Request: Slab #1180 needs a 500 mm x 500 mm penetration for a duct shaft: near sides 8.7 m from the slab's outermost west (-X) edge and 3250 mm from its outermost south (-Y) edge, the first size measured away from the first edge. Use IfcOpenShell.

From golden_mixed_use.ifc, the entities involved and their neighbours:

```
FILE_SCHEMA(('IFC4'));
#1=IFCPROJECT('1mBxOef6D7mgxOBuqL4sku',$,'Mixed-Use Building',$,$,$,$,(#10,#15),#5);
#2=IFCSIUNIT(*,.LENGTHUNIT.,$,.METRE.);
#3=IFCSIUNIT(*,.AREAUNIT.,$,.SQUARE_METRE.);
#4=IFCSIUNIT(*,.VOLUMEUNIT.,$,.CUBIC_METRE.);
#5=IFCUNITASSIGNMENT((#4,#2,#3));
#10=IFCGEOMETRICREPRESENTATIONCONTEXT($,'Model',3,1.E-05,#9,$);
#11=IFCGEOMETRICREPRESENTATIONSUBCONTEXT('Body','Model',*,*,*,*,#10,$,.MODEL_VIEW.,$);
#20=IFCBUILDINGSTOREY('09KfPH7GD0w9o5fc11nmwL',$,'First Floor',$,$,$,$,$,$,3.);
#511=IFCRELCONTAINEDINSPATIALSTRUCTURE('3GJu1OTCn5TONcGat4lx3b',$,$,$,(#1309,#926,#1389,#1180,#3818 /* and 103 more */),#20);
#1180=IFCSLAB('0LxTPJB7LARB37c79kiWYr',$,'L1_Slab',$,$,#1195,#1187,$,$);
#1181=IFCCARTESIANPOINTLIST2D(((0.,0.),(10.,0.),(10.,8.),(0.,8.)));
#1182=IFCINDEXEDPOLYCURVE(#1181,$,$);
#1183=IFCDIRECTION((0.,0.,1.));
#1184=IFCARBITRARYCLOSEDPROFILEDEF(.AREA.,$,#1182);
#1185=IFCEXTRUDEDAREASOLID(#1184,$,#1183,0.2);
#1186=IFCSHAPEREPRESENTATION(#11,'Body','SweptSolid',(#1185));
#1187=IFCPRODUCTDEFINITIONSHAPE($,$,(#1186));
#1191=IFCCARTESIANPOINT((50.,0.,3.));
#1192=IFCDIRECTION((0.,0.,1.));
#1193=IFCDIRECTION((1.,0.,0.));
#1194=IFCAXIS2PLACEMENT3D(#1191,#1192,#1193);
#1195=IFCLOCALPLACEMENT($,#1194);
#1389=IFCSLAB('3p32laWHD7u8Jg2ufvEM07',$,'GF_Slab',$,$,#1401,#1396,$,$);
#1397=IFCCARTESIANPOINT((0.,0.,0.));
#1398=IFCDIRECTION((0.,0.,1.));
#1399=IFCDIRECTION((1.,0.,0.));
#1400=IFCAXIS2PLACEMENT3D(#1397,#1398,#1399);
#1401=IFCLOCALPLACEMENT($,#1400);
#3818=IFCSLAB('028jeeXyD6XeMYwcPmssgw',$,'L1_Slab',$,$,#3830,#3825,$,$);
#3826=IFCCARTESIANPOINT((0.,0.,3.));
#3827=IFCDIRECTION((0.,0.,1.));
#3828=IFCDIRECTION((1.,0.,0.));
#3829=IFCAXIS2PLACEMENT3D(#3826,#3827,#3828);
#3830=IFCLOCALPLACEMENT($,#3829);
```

```python
import numpy as np
import ifcopenshell
import ifcopenshell.api.feature
import ifcopenshell.api.geometry
import ifcopenshell.api.root
import ifcopenshell.geom
import ifcopenshell.util.placement
import ifcopenshell.util.representation
import ifcopenshell.util.shape
import ifcopenshell.util.unit

model = ifcopenshell.open("golden_mixed_use.ifc")
unit_scale = ifcopenshell.util.unit.calculate_unit_scale(model)
settings = ifcopenshell.geom.settings()


def volume(element):
    """Net volume in cubic metres, openings subtracted."""
    shape = ifcopenshell.geom.create_shape(settings, element)
    return ifcopenshell.util.shape.get_volume(shape.geometry)


slab = model.by_guid("0LxTPJB7LARB37c79kiWYr")
before = volume(slab)

# Extent in the slab's own axes, in metres. The edges named are its -X and -Y sides.
slab_shape = ifcopenshell.geom.create_shape(settings, slab)
vertices = ifcopenshell.util.shape.get_vertices(slab_shape.geometry)
x_min, y_min, bottom = vertices.min(axis=0)
top = vertices[:, 2].max()

opening = ifcopenshell.api.root.create_entity(model, ifc_class="IfcOpeningElement", name="Duct shaft opening", predefined_type="OPENING")
context = ifcopenshell.util.representation.get_context(model, "Model", "Body", "MODEL_VIEW")
width, depth = 0.5, 0.5
outline = [(0.0, 0.0), (width, 0.0), (width, depth), (0.0, depth), (0.0, 0.0)]
# Overshoot both faces by 50 mm so the cut is clean.
shape = ifcopenshell.api.geometry.add_slab_representation(
    model, context=context, depth=top - bottom + 0.1, polyline=outline
)
ifcopenshell.api.geometry.assign_representation(model, product=opening, representation=shape)

matrix = ifcopenshell.util.placement.get_local_placement(slab.ObjectPlacement)
matrix[:, 3] = matrix @ np.append(np.array([x_min + 8.7, y_min + 3.25, bottom - 0.05]) / unit_scale, 1.0)
ifcopenshell.api.geometry.edit_object_placement(model, product=opening, matrix=matrix, is_si=False)
ifcopenshell.api.feature.add_feature(model, feature=opening, element=slab)

after = volume(slab)

print(f"slab volume {before:.3f} -> {after:.3f} m3")

model.write("golden_mixed_use_updated.ifc")
```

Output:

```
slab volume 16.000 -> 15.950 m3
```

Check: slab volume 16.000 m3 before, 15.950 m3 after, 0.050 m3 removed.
